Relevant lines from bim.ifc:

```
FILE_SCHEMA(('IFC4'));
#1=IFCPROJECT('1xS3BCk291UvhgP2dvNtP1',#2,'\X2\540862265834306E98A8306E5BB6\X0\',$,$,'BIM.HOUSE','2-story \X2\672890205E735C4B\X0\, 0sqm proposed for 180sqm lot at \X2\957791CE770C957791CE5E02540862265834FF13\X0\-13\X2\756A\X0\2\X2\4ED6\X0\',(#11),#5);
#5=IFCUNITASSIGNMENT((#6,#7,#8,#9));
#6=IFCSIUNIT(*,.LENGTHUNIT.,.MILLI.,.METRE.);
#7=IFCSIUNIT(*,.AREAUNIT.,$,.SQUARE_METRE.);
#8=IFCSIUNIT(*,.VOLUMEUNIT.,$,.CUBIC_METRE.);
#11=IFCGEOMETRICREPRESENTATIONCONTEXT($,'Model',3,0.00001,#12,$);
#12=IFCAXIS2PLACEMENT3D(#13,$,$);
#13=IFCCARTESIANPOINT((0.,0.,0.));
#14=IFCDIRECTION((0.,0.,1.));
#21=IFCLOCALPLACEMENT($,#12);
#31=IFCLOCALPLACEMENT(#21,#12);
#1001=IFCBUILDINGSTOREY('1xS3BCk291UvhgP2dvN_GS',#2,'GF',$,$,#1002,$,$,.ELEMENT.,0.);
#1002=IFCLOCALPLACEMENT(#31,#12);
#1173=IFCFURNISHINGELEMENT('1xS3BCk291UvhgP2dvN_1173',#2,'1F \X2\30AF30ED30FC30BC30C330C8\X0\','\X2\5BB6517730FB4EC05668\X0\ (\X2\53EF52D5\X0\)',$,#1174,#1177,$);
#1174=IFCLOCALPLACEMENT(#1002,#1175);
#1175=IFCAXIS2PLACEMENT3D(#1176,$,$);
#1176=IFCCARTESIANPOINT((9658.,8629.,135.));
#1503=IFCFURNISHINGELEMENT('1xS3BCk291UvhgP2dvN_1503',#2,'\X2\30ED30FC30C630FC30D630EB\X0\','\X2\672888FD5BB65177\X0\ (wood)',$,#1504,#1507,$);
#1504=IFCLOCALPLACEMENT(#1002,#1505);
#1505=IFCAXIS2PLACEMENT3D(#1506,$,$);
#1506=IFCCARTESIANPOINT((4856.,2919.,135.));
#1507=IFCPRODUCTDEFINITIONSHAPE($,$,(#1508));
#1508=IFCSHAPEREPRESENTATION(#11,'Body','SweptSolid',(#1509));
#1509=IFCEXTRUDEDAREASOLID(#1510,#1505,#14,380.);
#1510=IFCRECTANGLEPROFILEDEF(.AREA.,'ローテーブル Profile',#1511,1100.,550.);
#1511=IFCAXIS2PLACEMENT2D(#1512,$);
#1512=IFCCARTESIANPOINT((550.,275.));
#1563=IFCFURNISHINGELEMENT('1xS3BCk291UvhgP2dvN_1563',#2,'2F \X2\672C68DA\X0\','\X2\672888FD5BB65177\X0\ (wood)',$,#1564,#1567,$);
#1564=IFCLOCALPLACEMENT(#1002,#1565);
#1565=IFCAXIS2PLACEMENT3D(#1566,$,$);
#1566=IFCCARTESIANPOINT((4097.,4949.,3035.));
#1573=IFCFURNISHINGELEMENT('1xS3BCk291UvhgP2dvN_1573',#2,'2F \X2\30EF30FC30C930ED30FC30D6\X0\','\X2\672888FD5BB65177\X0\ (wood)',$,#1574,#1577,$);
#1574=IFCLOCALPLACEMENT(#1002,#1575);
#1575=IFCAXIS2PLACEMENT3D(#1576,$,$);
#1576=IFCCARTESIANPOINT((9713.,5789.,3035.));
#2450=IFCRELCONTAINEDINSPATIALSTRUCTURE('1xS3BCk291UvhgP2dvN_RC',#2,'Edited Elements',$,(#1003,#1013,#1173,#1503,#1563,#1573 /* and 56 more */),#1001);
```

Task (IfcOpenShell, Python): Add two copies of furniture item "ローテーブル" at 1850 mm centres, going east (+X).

```python
import numpy as np
import ifcopenshell
import ifcopenshell.api.geometry
import ifcopenshell.api.root
import ifcopenshell.util.element
import ifcopenshell.util.placement
import ifcopenshell.util.unit

model = ifcopenshell.open("bim.ifc")
unit_scale = ifcopenshell.util.unit.calculate_unit_scale(model)


def reuse_history(source, copy):
    """copy_class also copies each property set's owner history, people and application; keep the originals."""
    for rel in copy.IsDefinedBy:
        if rel.is_a("IfcRelDefinesByProperties") and (history := rel.RelatingPropertyDefinition.OwnerHistory):
            rel.RelatingPropertyDefinition.OwnerHistory = source.OwnerHistory
            ifcopenshell.util.element.remove_deep2(model, history)


source = model.by_guid("1xS3BCk291UvhgP2dvN_1503")
base = ifcopenshell.util.placement.get_local_placement(source.ObjectPlacement)
step = np.array([1.0, 0.0, 0.0]) * 1.85 / unit_scale

for i in range(1, 3):
    copy = ifcopenshell.api.root.copy_class(model, product=source)
    copy.Representation = ifcopenshell.util.element.copy_deep(
        model, source.Representation, exclude=["IfcGeometricRepresentationContext", "IfcRepresentationMap"]
    )
    reuse_history(source, copy)
    matrix = base.copy()
    matrix[:3, 3] += i * step
    print("added at", matrix[:3, 3].round(3) + 0.0)
    ifcopenshell.api.geometry.edit_object_placement(model, product=copy, matrix=matrix, is_si=False)

model.write("bim_rev.ifc")
```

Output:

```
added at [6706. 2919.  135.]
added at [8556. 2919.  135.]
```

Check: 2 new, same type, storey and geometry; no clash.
